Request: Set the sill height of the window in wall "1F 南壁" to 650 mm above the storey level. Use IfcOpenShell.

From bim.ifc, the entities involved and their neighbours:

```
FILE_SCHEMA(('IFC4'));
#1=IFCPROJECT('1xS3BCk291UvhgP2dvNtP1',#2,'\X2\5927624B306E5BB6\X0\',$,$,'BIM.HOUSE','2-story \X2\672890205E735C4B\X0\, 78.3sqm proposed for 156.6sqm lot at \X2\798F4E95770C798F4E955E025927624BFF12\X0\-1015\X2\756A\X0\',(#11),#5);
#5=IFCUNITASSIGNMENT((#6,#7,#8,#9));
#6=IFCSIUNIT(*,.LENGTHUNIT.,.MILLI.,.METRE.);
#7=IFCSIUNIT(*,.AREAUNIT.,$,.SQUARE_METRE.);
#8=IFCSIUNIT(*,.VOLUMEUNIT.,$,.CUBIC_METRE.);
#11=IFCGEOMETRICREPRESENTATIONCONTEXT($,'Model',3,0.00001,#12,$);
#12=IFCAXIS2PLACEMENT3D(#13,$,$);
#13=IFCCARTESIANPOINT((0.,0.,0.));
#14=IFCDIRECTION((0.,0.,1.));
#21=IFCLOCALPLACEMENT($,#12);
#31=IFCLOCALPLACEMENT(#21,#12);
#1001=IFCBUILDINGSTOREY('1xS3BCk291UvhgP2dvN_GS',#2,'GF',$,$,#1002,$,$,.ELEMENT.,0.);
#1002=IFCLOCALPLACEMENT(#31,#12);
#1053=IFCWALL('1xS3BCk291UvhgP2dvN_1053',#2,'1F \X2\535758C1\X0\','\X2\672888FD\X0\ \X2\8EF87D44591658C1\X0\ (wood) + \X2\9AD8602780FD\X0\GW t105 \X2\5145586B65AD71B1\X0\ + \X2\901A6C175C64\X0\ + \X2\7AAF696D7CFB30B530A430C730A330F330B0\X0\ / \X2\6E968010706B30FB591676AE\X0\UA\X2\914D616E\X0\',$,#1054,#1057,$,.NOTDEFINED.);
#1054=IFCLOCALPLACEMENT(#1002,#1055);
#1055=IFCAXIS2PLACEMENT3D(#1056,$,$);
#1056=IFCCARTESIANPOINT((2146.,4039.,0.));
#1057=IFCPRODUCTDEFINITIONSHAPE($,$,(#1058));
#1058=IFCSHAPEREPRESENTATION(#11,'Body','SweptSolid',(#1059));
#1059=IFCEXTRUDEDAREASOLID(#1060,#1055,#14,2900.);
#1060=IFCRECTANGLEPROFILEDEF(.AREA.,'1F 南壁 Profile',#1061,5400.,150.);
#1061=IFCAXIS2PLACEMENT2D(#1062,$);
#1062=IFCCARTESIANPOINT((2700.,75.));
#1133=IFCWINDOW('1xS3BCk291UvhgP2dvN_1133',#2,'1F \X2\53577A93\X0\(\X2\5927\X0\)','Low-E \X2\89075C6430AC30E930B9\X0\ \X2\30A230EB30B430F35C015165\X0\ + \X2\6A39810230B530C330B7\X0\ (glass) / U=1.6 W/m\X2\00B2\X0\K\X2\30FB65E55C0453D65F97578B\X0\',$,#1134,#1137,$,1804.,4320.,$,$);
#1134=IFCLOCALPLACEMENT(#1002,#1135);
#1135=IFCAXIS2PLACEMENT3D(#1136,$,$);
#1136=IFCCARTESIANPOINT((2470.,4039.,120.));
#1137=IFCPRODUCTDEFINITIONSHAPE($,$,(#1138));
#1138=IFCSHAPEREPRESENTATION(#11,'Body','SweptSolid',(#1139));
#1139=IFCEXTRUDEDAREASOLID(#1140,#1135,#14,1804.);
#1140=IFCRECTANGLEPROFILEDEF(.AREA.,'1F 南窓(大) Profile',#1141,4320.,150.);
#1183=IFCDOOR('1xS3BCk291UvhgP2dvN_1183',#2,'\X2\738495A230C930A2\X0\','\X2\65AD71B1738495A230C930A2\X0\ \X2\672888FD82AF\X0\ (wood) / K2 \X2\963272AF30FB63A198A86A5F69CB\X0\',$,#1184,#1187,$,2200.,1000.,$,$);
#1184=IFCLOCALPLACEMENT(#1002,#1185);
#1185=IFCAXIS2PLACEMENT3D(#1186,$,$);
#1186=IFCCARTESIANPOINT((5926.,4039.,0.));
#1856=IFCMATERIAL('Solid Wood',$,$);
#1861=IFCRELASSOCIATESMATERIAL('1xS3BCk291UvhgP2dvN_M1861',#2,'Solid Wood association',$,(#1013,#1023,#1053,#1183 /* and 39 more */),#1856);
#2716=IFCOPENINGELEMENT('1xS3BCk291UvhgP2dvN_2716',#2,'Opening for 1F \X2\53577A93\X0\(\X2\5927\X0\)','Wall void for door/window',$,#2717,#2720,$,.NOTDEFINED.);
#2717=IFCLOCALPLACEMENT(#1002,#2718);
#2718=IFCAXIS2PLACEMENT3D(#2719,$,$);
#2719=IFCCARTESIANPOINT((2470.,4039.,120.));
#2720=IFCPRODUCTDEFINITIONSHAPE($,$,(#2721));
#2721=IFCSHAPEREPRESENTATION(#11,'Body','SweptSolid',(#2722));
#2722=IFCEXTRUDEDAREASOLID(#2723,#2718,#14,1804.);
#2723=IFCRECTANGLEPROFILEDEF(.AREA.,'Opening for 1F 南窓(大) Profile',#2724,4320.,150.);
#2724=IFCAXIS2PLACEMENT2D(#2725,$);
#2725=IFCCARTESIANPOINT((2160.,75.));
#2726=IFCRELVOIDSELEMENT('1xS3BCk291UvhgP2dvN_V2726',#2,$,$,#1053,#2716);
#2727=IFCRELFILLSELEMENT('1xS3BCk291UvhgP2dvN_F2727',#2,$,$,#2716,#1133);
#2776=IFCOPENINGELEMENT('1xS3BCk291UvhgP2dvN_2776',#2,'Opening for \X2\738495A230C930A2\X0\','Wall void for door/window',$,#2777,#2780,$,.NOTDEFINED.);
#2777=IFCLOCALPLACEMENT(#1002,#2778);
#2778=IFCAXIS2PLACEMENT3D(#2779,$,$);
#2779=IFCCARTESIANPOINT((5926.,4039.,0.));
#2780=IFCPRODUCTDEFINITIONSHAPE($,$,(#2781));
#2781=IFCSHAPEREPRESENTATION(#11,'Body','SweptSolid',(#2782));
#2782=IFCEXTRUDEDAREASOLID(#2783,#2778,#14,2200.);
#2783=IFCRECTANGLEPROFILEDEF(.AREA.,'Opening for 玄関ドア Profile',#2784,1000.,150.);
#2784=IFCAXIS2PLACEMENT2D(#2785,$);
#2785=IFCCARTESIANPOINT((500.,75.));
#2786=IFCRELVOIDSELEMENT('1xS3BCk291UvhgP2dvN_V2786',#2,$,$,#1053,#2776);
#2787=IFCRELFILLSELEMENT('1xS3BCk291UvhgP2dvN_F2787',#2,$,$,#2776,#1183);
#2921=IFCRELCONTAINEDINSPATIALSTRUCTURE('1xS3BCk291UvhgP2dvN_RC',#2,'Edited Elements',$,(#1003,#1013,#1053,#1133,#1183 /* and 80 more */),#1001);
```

```python
import numpy as np
import ifcopenshell
import ifcopenshell.api.geometry
import ifcopenshell.geom
import ifcopenshell.util.element
import ifcopenshell.util.placement
import ifcopenshell.util.shape
import ifcopenshell.util.unit

model = ifcopenshell.open("bim.ifc")
unit_scale = ifcopenshell.util.unit.calculate_unit_scale(model)

window = model.by_id(1133)
opening = window.FillsVoids[0].RelatingOpeningElement
storey = ifcopenshell.util.element.get_container(window, ifc_class="IfcBuildingStorey")
level = ifcopenshell.util.placement.get_local_placement(storey.ObjectPlacement)[2, 3]

# The opening's origin need not be at the sill, so measure its lowest point.
shape = ifcopenshell.geom.create_shape(ifcopenshell.geom.settings(), opening)
bottom = ifcopenshell.util.shape.get_shape_bottom_elevation(shape, shape.geometry) / unit_scale
dz = level + 0.65 / unit_scale - bottom

shift = np.array([0.0, 0.0, dz])
# The window is not placed relative to its opening, so move both.
for product in (opening, window):
    matrix = ifcopenshell.util.placement.get_local_placement(product.ObjectPlacement)
    matrix[:3, 3] += shift
    ifcopenshell.api.geometry.edit_object_placement(model, product=product, matrix=matrix, is_si=False)

print(f"moved by {dz * unit_scale:+.3f} m")

model.write("bim_edited.ifc")
```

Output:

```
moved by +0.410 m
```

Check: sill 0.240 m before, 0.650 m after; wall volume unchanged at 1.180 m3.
